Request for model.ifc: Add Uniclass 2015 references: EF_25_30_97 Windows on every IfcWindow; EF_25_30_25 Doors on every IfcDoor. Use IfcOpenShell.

First a look at what the model holds.

```python
import ifcopenshell

model = ifcopenshell.open("model.ifc")
print(model.schema)
print("classifications:", [c.Name for c in model.by_type("IfcClassification")])
for ifc_class in ("IfcDoor", "IfcRoof", "IfcStair", "IfcWall", "IfcWindow"):
    print(ifc_class, len(model.by_type(ifc_class)))
```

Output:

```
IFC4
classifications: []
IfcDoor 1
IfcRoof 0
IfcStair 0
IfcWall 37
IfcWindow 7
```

```python
import ifcopenshell
import ifcopenshell.api.classification

model = ifcopenshell.open("model.ifc")

system = ifcopenshell.api.classification.add_classification(model, classification="Uniclass 2015")

codes = {
    "IfcWindow": ("EF_25_30_97", "Windows"),
    "IfcDoor": ("EF_25_30_25", "Doors"),
}
for ifc_class, (code, name) in codes.items():
    products = model.by_type(ifc_class)
    ifcopenshell.api.classification.add_reference(
        model, products=products, classification=system, identification=code, name=name
    )
    print(code, len(products))

model.write("model_updated.ifc")
```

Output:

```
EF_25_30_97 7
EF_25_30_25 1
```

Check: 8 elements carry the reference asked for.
